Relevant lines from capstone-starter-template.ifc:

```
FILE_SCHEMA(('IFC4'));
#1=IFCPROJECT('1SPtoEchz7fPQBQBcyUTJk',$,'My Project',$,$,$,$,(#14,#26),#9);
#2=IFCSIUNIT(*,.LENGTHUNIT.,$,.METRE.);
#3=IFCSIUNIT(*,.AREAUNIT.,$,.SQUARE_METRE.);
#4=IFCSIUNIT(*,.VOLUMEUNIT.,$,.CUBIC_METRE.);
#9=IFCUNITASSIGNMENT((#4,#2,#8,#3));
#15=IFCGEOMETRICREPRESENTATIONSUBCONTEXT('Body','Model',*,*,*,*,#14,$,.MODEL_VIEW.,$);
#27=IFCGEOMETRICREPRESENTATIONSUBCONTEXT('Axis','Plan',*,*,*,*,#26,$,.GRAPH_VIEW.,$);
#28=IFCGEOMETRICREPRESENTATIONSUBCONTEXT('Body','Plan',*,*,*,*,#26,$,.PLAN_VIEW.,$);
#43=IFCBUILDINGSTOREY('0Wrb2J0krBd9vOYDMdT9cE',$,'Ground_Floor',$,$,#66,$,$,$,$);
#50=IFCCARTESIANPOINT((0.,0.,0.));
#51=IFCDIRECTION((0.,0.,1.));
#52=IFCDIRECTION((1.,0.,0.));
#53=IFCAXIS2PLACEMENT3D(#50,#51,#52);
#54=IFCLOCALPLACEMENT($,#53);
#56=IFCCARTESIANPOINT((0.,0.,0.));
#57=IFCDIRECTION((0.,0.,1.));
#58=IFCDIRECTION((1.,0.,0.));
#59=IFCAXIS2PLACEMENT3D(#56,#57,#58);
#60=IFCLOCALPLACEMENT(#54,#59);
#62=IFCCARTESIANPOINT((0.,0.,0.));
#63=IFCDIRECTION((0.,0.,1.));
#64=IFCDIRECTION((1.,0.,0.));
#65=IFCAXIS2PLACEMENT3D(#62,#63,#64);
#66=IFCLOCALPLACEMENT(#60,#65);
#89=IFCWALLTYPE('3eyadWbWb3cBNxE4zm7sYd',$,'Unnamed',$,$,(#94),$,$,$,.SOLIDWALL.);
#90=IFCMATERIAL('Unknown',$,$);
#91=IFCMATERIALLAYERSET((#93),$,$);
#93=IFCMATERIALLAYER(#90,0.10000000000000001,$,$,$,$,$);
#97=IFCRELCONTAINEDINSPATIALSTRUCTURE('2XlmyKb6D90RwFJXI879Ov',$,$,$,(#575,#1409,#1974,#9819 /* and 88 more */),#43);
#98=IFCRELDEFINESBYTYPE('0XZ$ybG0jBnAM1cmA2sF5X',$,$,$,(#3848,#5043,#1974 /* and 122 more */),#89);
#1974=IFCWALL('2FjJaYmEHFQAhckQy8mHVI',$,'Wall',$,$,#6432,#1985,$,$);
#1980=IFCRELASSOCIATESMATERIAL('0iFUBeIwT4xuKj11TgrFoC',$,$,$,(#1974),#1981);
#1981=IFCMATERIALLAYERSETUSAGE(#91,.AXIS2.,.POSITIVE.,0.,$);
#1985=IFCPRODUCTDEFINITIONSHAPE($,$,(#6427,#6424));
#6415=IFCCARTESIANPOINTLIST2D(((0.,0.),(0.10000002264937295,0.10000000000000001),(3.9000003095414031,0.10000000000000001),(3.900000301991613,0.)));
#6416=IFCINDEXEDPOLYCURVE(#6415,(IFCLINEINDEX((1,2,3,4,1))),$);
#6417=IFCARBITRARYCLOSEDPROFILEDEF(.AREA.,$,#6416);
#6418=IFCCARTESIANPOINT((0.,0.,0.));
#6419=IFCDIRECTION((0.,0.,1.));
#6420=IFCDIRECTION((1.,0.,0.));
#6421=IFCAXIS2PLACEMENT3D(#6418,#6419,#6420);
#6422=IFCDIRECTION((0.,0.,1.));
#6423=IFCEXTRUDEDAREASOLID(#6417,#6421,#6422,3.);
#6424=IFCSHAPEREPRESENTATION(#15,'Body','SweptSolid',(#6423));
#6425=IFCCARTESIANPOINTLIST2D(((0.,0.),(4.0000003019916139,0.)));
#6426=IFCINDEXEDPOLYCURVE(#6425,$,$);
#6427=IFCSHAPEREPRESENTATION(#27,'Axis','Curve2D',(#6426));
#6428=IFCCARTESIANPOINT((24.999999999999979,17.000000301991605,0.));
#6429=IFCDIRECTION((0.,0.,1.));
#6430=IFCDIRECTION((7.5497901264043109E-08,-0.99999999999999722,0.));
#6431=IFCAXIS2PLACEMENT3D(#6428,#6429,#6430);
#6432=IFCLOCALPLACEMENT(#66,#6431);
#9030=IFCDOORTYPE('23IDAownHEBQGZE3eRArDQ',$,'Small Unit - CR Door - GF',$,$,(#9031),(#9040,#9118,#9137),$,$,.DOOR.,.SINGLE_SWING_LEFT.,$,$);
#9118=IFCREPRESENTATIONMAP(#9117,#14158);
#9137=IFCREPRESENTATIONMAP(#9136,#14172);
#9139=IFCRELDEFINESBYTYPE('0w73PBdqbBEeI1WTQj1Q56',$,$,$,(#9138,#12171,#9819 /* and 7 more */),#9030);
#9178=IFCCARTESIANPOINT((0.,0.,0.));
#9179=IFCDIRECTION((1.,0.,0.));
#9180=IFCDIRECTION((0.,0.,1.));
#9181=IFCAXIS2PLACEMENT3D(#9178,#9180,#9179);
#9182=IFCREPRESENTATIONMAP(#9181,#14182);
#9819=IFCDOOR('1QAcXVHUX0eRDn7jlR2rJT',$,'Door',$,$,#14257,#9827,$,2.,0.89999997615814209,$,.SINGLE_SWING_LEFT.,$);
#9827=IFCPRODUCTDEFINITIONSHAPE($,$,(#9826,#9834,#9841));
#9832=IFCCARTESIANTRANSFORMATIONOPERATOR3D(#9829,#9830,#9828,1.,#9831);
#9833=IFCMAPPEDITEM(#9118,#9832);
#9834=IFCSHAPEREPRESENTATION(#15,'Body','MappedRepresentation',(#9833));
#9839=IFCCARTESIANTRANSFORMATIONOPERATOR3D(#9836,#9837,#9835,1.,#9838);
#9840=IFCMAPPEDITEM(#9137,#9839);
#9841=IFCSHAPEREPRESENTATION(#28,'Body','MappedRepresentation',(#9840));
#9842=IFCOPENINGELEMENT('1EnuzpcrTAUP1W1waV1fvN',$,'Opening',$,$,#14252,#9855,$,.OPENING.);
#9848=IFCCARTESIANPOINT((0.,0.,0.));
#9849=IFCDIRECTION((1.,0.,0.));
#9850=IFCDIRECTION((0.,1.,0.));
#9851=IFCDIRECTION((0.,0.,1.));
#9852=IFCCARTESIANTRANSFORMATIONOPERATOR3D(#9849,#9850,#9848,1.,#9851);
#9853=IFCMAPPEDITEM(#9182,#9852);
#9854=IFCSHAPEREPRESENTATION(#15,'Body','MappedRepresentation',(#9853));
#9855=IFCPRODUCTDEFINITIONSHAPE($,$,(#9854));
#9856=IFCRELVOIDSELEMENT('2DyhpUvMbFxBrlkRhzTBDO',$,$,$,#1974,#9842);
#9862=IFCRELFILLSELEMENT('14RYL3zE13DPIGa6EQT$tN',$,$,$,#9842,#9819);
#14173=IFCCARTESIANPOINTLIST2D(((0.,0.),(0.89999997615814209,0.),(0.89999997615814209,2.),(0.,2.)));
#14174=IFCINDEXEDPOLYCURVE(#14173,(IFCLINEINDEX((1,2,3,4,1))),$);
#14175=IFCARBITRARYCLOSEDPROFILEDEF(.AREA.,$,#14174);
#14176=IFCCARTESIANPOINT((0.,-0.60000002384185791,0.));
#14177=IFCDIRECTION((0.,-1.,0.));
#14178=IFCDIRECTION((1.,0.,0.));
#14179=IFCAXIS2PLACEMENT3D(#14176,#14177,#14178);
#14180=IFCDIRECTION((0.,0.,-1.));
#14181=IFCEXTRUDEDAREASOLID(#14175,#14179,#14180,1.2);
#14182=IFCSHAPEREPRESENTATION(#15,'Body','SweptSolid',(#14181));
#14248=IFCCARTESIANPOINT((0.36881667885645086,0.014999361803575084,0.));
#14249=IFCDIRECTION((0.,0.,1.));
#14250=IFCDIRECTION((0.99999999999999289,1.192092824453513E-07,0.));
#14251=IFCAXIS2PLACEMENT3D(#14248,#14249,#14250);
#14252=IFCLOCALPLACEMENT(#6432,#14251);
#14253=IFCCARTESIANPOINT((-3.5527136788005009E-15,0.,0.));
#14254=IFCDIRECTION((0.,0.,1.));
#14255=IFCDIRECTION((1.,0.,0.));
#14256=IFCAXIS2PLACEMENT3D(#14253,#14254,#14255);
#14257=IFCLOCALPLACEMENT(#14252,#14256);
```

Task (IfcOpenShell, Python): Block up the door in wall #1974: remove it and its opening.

```python
import ifcopenshell
import ifcopenshell.api.feature
import ifcopenshell.api.root
import ifcopenshell.geom
import ifcopenshell.util.shape

model = ifcopenshell.open("capstone-starter-template.ifc")
settings = ifcopenshell.geom.settings()


def volume(element):
    """Net volume in cubic metres, openings subtracted."""
    shape = ifcopenshell.geom.create_shape(settings, element)
    return ifcopenshell.util.shape.get_volume(shape.geometry)


door = model.by_guid("1QAcXVHUX0eRDn7jlR2rJT")
opening = door.FillsVoids[0].RelatingOpeningElement
wall = opening.VoidsElements[0].RelatingBuildingElement
before = volume(wall)

ifcopenshell.api.root.remove_product(model, product=door)
ifcopenshell.api.feature.remove_feature(model, feature=opening)

after = volume(wall)

print(f"wall volume {before:.3f} -> {after:.3f} m3")

model.write("capstone-starter-template-out.ifc")
```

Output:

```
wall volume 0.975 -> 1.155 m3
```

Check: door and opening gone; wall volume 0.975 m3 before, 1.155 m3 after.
